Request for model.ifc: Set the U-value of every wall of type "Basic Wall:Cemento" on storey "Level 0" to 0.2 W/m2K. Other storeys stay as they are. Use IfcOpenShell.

First a look at what the model holds.

```python
import ifcopenshell
import ifcopenshell.util.element

model = ifcopenshell.open("model.ifc")
print(model.schema)
storey = next(s for s in model.by_type("IfcBuildingStorey") if s.Name == "Level 0")
walls = [e for e in ifcopenshell.util.element.get_decomposition(storey) if e.is_a("IfcWall")]
seen = {}
for e in walls:
    element_type = ifcopenshell.util.element.get_type(e)
    key = (element_type.Name if element_type != e and element_type else None, ifcopenshell.util.element.get_pset(e, "Pset_WallCommon", "ThermalTransmittance"))
    seen[key] = seen.get(key, 0) + 1
for (name, value), count in sorted(seen.items(), key=str):
    print(count, "x", name, "|", value)
```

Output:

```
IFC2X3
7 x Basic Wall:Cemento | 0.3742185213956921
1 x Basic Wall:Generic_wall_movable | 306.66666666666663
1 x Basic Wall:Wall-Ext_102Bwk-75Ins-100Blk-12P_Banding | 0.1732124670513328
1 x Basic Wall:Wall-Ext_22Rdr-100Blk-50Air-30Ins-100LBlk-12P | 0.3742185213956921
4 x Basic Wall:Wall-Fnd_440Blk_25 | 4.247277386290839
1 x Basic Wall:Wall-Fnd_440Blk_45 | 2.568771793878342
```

```python
import ifcopenshell
import ifcopenshell.api.pset
import ifcopenshell.util.element

model = ifcopenshell.open("model.ifc")

storey = next(s for s in model.by_type("IfcBuildingStorey") if s.Name == "Level 0")
walls = [e for e in ifcopenshell.util.element.get_decomposition(storey) if e.is_a("IfcWall")]

count = 0
for e in walls:
    element_type = ifcopenshell.util.element.get_type(e)
    if element_type in (None, e) or element_type.Name != "Basic Wall:Cemento":
        continue
    # add_pset returns the element's existing set when there is one.
    pset = ifcopenshell.api.pset.add_pset(model, product=e, name="Pset_WallCommon")
    ifcopenshell.api.pset.edit_pset(model, pset=pset, properties={"ThermalTransmittance": 0.2})
    count += 1

print(count, "walls updated")

model.write("model_updated.ifc")
```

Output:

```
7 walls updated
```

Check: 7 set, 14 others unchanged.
